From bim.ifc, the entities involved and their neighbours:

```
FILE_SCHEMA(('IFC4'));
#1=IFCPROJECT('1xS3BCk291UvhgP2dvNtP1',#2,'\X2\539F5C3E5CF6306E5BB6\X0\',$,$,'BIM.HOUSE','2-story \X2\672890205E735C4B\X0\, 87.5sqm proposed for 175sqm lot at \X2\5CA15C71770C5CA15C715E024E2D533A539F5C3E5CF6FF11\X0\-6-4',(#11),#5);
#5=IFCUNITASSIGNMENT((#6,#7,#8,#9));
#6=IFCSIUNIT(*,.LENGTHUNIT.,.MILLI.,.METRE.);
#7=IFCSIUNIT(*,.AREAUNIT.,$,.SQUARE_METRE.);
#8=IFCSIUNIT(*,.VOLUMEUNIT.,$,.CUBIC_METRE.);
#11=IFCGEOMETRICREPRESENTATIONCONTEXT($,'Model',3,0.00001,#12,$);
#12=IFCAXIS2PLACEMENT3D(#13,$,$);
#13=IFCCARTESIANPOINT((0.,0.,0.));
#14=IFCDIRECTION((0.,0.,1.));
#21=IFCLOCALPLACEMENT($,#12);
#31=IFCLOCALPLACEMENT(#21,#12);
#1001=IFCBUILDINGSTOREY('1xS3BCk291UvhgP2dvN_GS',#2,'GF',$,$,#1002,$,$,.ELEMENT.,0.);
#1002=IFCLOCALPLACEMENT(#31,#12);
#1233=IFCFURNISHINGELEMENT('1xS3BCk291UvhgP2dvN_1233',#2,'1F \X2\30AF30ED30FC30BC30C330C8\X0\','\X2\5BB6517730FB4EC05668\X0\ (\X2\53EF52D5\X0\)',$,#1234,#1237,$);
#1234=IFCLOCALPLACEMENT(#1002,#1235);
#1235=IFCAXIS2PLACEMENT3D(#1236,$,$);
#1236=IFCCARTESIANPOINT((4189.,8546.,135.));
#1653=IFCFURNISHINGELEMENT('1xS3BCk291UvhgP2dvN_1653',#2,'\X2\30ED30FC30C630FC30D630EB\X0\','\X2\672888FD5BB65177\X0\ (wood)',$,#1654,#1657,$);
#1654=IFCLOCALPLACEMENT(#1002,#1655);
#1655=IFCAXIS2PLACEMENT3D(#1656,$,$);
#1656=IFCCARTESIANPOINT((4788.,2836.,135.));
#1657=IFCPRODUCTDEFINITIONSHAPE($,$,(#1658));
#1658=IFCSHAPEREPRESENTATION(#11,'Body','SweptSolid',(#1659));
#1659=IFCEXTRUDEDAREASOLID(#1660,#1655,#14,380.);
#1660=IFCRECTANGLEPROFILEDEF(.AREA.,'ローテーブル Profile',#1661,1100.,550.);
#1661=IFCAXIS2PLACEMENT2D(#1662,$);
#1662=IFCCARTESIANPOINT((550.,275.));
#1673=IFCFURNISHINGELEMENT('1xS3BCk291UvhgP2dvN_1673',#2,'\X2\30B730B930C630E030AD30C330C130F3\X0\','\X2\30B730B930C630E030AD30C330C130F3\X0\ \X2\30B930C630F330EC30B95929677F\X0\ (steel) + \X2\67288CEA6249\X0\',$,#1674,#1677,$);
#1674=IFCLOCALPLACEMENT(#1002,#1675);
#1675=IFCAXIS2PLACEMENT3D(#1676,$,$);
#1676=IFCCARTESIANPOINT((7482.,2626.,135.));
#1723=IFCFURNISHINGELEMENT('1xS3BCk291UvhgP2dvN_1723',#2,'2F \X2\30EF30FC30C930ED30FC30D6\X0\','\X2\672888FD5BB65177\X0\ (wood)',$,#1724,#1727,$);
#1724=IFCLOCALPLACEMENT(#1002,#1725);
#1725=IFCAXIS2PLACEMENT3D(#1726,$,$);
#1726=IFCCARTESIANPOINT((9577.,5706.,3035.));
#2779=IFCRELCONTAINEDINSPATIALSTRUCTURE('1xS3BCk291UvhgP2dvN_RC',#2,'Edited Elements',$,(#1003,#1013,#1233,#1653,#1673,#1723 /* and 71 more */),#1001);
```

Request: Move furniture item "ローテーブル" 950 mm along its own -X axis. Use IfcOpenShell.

```python
import ifcopenshell
import ifcopenshell.api.geometry
import ifcopenshell.util.placement

model = ifcopenshell.open("bim.ifc")

item = model.by_guid("1xS3BCk291UvhgP2dvN_1653")
matrix = ifcopenshell.util.placement.get_local_placement(item.ObjectPlacement)
matrix[:3, 3] -= matrix[:3, 0] * 950.0
ifcopenshell.api.geometry.edit_object_placement(model, product=item, matrix=matrix, is_si=False)

print(ifcopenshell.util.placement.get_local_placement(item.ObjectPlacement).round(3) + 0.0)

model.write("bim-out.ifc")
```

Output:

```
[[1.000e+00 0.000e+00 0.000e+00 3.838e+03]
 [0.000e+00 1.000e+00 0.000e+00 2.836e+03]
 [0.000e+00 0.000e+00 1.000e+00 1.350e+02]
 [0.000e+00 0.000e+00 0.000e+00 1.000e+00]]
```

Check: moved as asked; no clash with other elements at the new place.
